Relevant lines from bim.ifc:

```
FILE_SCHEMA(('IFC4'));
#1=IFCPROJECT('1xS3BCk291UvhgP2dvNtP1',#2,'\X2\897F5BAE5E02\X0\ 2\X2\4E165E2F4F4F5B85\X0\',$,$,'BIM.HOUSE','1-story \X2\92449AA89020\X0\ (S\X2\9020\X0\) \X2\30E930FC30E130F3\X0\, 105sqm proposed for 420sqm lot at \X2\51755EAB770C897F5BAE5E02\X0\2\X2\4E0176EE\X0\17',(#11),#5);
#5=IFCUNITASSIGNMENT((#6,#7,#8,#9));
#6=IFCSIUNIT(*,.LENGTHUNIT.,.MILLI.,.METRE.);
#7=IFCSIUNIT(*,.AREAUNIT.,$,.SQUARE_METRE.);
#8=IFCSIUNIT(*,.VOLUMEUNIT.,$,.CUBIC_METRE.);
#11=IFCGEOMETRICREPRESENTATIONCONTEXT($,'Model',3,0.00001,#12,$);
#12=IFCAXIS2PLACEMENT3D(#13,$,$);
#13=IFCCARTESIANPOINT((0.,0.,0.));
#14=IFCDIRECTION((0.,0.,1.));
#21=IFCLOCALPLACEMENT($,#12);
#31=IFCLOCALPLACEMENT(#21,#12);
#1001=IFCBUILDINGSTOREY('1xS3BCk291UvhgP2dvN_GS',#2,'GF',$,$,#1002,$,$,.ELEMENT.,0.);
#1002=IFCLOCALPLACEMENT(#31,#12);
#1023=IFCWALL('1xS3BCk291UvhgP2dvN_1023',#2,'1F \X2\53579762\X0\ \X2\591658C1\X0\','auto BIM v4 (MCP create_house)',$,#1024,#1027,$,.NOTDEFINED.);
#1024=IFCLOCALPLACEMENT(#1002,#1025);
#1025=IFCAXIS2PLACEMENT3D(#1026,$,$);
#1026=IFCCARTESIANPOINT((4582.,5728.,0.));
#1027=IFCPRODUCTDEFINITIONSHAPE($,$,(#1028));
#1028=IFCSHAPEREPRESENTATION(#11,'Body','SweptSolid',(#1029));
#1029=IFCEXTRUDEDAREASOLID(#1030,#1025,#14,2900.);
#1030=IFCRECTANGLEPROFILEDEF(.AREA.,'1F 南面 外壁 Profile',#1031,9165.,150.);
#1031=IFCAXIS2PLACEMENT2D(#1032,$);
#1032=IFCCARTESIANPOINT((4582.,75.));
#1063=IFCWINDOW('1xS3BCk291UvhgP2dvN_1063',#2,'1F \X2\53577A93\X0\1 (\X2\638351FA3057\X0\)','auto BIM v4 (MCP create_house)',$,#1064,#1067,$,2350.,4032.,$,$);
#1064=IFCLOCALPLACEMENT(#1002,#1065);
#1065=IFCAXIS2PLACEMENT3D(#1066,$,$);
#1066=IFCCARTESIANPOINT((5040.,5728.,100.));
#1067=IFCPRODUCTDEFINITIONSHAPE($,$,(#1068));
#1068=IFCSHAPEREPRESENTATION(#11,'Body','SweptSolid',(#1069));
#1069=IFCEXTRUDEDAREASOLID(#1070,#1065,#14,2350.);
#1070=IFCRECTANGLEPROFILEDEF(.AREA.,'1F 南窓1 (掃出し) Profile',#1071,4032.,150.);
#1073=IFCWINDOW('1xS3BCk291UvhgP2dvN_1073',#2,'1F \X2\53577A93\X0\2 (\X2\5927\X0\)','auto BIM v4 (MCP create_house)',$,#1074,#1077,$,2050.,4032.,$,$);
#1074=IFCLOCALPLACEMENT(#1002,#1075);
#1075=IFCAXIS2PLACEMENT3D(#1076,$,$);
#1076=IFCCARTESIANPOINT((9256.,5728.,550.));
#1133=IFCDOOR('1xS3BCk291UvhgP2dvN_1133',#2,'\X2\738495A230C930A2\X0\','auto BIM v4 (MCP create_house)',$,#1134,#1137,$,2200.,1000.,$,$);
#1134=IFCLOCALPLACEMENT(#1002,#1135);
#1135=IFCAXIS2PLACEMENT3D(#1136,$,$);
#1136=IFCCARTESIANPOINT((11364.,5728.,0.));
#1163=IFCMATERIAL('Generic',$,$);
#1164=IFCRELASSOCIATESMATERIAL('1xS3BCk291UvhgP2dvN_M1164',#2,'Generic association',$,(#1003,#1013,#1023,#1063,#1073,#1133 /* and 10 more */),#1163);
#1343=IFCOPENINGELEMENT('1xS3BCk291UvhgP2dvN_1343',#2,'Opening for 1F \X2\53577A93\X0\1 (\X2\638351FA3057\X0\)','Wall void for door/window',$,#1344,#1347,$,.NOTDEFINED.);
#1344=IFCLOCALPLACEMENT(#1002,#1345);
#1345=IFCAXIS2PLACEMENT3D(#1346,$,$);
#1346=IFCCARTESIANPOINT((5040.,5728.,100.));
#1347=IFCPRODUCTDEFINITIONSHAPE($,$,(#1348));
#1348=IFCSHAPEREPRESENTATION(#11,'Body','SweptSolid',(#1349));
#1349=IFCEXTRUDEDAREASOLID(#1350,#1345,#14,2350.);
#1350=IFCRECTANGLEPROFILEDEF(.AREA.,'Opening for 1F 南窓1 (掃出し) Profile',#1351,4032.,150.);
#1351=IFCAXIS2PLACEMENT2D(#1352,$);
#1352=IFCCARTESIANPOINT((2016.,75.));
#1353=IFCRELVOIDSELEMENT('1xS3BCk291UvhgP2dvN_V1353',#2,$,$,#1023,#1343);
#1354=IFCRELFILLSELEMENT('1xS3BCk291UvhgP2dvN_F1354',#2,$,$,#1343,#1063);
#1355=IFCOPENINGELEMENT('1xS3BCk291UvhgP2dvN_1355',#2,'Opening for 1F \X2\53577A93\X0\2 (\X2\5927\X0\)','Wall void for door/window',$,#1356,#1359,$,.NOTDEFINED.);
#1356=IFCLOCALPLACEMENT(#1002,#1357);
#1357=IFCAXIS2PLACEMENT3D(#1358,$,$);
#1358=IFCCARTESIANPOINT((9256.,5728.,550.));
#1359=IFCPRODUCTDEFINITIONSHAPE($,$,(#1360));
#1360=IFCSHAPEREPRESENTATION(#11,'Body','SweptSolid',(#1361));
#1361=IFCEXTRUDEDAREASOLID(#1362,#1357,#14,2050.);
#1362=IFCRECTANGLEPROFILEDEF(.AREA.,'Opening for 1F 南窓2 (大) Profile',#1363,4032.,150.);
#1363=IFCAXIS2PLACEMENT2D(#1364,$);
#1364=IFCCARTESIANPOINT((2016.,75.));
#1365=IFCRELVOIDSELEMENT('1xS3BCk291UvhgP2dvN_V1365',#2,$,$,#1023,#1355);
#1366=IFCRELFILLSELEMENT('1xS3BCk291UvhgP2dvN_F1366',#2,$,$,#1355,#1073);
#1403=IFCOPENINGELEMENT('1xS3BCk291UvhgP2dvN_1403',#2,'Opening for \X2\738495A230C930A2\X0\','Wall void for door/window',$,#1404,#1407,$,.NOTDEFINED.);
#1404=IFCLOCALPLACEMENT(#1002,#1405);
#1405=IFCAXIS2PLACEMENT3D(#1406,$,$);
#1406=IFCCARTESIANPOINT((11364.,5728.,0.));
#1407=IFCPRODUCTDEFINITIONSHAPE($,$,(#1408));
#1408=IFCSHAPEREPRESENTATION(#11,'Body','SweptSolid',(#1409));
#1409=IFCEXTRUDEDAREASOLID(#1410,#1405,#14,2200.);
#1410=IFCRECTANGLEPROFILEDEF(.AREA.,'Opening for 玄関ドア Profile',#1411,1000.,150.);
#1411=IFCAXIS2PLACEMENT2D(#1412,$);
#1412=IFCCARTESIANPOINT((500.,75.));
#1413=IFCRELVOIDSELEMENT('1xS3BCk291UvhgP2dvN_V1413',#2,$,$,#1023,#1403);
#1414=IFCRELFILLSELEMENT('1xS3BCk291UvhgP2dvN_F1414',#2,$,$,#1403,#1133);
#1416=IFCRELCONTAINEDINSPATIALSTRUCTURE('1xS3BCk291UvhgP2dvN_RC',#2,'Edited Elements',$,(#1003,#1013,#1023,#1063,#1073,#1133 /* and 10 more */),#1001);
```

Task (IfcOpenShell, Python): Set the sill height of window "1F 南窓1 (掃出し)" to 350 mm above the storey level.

```python
import numpy as np
import ifcopenshell
import ifcopenshell.api.geometry
import ifcopenshell.geom
import ifcopenshell.util.element
import ifcopenshell.util.placement
import ifcopenshell.util.shape
import ifcopenshell.util.unit

model = ifcopenshell.open("bim.ifc")
unit_scale = ifcopenshell.util.unit.calculate_unit_scale(model)

window = model.by_guid("1xS3BCk291UvhgP2dvN_1063")
opening = window.FillsVoids[0].RelatingOpeningElement
storey = ifcopenshell.util.element.get_container(window, ifc_class="IfcBuildingStorey")
level = ifcopenshell.util.placement.get_local_placement(storey.ObjectPlacement)[2, 3]

# The opening's origin need not be at the sill, so measure its lowest point.
shape = ifcopenshell.geom.create_shape(ifcopenshell.geom.settings(), opening)
bottom = ifcopenshell.util.shape.get_shape_bottom_elevation(shape, shape.geometry) / unit_scale
dz = level + 350.0 - bottom

shift = np.array([0.0, 0.0, dz])
# The window is not placed relative to its opening, so move both.
for product in (opening, window):
    matrix = ifcopenshell.util.placement.get_local_placement(product.ObjectPlacement)
    matrix[:3, 3] += shift
    ifcopenshell.api.geometry.edit_object_placement(model, product=product, matrix=matrix, is_si=False)

print(f"moved by {dz * unit_scale:+.3f} m")

model.write("bim_updated.ifc")
```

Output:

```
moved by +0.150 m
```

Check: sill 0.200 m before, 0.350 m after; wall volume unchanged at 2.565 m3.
